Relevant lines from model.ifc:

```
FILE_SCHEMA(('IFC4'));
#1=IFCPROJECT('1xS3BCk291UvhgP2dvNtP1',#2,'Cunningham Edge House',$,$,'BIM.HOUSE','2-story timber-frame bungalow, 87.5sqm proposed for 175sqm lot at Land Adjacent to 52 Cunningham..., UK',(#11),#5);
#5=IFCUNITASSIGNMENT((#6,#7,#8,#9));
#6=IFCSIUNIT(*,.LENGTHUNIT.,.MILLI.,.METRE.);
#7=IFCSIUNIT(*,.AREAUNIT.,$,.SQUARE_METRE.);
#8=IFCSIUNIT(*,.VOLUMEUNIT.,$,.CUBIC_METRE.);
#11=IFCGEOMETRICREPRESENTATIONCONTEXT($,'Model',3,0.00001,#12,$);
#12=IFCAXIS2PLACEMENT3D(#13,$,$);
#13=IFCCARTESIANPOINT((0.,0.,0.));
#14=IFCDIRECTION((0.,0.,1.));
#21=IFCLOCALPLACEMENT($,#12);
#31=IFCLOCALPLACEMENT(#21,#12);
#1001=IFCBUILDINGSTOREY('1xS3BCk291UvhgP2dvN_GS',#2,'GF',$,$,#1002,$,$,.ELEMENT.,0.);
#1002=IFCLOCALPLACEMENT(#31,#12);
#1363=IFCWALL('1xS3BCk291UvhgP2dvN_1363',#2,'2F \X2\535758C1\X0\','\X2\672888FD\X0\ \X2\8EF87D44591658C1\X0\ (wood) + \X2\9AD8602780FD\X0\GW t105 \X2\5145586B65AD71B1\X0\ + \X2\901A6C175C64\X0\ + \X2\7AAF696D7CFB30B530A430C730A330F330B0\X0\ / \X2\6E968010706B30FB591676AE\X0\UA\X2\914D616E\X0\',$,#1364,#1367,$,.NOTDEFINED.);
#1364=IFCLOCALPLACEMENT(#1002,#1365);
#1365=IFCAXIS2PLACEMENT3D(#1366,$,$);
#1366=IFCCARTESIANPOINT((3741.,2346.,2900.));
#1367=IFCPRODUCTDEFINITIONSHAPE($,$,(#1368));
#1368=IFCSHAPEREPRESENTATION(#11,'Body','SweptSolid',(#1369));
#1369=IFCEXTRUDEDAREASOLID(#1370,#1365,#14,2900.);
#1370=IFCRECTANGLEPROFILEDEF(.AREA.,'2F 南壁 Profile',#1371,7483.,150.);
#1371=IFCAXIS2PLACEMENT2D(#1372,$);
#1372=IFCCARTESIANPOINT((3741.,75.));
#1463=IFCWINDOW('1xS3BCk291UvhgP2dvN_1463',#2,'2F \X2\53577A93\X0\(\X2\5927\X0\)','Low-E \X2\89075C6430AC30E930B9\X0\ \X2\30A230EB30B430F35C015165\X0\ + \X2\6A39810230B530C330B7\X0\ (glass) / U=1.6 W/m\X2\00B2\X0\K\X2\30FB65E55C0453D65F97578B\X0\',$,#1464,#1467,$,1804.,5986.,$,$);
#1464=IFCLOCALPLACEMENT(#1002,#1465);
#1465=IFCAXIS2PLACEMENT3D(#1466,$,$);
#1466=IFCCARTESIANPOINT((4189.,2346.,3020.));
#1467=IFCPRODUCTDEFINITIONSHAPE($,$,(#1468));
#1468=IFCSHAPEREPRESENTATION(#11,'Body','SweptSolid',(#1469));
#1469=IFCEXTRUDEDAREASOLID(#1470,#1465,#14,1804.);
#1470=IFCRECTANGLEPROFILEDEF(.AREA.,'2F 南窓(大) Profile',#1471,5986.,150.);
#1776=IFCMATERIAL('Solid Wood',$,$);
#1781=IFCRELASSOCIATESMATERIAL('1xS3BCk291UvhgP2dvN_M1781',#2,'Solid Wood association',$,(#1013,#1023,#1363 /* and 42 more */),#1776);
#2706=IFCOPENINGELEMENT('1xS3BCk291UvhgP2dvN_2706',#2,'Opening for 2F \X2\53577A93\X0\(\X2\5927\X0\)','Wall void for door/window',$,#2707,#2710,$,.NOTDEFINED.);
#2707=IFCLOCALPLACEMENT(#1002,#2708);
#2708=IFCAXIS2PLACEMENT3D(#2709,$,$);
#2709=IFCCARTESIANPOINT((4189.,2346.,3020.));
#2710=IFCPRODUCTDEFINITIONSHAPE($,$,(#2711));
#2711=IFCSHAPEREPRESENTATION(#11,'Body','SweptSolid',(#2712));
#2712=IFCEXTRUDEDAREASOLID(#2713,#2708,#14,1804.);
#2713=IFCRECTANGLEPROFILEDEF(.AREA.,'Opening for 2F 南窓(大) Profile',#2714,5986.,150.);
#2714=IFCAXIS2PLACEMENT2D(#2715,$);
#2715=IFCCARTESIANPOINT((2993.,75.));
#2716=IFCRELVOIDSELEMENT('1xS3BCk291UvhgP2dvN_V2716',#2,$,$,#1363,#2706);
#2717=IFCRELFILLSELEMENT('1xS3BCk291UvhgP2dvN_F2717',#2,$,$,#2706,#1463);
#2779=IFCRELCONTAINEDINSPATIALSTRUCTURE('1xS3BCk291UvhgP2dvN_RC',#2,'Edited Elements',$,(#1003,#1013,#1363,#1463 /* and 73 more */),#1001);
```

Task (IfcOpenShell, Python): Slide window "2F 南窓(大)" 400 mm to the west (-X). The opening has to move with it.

```python
import ifcopenshell
import ifcopenshell.api.geometry
import ifcopenshell.util.placement
import ifcopenshell.util.unit

model = ifcopenshell.open("model.ifc")
unit_scale = ifcopenshell.util.unit.calculate_unit_scale(model)

window = model.by_guid("1xS3BCk291UvhgP2dvN_1463")
opening = window.FillsVoids[0].RelatingOpeningElement
wall = opening.VoidsElements[0].RelatingBuildingElement

wall_matrix = ifcopenshell.util.placement.get_local_placement(wall.ObjectPlacement)
shift = wall_matrix[:3, 0] * -0.4 / unit_scale
before = ifcopenshell.util.placement.get_local_placement(window.ObjectPlacement)[:3, 3].copy()

# The window is not placed relative to its opening, so move both.
for product in (opening, window):
    matrix = ifcopenshell.util.placement.get_local_placement(product.ObjectPlacement)
    matrix[:3, 3] += shift
    ifcopenshell.api.geometry.edit_object_placement(model, product=product, matrix=matrix, is_si=False)

after = ifcopenshell.util.placement.get_local_placement(window.ObjectPlacement)[:3, 3]
print("window moved by", (after - before).round(3) + 0.0)

model.write("model_v2.ifc")
```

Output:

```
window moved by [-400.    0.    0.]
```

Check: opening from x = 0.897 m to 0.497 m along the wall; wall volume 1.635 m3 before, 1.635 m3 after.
